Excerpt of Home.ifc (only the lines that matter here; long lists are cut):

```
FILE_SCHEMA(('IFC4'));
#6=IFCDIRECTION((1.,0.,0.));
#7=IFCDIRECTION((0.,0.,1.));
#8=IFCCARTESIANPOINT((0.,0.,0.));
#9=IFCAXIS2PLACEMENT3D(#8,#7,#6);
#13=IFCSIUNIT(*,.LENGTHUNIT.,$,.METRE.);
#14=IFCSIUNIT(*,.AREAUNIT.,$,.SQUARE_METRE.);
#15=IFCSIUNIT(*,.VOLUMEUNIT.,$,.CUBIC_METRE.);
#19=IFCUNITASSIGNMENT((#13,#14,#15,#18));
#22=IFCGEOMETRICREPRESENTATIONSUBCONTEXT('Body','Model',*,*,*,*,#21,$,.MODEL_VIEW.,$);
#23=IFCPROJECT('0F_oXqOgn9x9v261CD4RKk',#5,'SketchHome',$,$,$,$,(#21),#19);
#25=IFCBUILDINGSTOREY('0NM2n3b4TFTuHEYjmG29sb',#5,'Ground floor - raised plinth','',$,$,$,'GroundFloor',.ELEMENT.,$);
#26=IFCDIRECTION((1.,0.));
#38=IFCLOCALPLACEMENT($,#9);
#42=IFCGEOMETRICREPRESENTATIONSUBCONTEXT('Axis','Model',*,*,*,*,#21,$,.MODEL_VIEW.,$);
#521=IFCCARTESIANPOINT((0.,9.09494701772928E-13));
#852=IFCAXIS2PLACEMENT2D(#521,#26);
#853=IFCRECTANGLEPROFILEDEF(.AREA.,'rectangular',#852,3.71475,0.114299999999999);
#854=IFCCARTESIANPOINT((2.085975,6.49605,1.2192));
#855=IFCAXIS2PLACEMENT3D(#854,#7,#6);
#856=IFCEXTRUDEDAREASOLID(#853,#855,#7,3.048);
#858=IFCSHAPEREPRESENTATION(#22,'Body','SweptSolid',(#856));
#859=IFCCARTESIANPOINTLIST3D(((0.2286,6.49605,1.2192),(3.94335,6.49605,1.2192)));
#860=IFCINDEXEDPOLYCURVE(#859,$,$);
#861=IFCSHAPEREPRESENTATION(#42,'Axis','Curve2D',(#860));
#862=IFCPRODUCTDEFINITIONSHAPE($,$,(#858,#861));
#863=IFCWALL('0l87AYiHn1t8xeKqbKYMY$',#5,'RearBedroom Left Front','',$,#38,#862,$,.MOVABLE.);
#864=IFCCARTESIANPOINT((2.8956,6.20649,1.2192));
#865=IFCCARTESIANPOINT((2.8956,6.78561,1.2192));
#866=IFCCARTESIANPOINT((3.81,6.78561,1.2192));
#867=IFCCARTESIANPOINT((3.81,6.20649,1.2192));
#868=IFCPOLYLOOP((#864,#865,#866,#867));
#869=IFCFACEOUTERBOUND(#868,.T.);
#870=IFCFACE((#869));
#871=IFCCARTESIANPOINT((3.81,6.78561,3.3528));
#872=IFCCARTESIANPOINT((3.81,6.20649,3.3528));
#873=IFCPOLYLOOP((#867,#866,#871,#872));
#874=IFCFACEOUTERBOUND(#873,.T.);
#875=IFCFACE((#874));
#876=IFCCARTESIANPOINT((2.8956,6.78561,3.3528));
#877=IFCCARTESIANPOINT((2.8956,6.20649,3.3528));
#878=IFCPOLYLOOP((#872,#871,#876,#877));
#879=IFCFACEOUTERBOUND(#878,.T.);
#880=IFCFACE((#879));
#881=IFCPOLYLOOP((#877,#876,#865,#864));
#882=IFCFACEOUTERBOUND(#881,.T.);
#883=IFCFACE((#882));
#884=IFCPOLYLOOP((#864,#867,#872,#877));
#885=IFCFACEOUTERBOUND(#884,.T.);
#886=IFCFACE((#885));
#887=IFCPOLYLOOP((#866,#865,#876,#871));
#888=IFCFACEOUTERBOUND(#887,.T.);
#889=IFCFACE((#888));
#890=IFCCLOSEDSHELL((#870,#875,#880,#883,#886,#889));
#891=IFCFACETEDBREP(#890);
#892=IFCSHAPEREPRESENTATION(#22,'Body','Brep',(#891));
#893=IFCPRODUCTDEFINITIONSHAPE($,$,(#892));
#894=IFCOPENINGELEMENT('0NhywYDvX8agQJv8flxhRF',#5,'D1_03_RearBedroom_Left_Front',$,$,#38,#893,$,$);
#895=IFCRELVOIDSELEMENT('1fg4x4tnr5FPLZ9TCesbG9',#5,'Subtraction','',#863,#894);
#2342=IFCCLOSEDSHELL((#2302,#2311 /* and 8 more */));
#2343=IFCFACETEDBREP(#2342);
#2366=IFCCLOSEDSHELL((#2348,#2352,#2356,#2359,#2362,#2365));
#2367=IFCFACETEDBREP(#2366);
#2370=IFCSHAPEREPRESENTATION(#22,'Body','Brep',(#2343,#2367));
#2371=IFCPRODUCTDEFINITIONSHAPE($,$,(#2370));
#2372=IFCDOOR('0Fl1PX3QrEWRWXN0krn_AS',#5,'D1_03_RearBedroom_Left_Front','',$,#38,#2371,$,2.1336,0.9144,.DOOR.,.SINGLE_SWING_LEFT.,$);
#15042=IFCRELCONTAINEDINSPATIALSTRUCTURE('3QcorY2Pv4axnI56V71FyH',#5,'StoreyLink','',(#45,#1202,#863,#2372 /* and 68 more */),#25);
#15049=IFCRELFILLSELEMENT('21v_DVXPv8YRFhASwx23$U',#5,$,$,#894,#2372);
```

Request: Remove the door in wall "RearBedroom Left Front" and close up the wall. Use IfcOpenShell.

```python
import ifcopenshell
import ifcopenshell.api.feature
import ifcopenshell.api.root
import ifcopenshell.geom
import ifcopenshell.util.shape

model = ifcopenshell.open("Home.ifc")
settings = ifcopenshell.geom.settings()


def volume(element):
    """Net volume in cubic metres, openings subtracted."""
    shape = ifcopenshell.geom.create_shape(settings, element)
    return ifcopenshell.util.shape.get_volume(shape.geometry)


door = model.by_guid("0Fl1PX3QrEWRWXN0krn_AS")
opening = door.FillsVoids[0].RelatingOpeningElement
wall = opening.VoidsElements[0].RelatingBuildingElement
before = volume(wall)

ifcopenshell.api.root.remove_product(model, product=door)
ifcopenshell.api.feature.remove_feature(model, feature=opening)

after = volume(wall)

print(f"wall volume {before:.3f} -> {after:.3f} m3")

model.write("Home-out.ifc")
```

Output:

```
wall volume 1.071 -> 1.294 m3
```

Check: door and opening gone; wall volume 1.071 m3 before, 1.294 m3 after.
